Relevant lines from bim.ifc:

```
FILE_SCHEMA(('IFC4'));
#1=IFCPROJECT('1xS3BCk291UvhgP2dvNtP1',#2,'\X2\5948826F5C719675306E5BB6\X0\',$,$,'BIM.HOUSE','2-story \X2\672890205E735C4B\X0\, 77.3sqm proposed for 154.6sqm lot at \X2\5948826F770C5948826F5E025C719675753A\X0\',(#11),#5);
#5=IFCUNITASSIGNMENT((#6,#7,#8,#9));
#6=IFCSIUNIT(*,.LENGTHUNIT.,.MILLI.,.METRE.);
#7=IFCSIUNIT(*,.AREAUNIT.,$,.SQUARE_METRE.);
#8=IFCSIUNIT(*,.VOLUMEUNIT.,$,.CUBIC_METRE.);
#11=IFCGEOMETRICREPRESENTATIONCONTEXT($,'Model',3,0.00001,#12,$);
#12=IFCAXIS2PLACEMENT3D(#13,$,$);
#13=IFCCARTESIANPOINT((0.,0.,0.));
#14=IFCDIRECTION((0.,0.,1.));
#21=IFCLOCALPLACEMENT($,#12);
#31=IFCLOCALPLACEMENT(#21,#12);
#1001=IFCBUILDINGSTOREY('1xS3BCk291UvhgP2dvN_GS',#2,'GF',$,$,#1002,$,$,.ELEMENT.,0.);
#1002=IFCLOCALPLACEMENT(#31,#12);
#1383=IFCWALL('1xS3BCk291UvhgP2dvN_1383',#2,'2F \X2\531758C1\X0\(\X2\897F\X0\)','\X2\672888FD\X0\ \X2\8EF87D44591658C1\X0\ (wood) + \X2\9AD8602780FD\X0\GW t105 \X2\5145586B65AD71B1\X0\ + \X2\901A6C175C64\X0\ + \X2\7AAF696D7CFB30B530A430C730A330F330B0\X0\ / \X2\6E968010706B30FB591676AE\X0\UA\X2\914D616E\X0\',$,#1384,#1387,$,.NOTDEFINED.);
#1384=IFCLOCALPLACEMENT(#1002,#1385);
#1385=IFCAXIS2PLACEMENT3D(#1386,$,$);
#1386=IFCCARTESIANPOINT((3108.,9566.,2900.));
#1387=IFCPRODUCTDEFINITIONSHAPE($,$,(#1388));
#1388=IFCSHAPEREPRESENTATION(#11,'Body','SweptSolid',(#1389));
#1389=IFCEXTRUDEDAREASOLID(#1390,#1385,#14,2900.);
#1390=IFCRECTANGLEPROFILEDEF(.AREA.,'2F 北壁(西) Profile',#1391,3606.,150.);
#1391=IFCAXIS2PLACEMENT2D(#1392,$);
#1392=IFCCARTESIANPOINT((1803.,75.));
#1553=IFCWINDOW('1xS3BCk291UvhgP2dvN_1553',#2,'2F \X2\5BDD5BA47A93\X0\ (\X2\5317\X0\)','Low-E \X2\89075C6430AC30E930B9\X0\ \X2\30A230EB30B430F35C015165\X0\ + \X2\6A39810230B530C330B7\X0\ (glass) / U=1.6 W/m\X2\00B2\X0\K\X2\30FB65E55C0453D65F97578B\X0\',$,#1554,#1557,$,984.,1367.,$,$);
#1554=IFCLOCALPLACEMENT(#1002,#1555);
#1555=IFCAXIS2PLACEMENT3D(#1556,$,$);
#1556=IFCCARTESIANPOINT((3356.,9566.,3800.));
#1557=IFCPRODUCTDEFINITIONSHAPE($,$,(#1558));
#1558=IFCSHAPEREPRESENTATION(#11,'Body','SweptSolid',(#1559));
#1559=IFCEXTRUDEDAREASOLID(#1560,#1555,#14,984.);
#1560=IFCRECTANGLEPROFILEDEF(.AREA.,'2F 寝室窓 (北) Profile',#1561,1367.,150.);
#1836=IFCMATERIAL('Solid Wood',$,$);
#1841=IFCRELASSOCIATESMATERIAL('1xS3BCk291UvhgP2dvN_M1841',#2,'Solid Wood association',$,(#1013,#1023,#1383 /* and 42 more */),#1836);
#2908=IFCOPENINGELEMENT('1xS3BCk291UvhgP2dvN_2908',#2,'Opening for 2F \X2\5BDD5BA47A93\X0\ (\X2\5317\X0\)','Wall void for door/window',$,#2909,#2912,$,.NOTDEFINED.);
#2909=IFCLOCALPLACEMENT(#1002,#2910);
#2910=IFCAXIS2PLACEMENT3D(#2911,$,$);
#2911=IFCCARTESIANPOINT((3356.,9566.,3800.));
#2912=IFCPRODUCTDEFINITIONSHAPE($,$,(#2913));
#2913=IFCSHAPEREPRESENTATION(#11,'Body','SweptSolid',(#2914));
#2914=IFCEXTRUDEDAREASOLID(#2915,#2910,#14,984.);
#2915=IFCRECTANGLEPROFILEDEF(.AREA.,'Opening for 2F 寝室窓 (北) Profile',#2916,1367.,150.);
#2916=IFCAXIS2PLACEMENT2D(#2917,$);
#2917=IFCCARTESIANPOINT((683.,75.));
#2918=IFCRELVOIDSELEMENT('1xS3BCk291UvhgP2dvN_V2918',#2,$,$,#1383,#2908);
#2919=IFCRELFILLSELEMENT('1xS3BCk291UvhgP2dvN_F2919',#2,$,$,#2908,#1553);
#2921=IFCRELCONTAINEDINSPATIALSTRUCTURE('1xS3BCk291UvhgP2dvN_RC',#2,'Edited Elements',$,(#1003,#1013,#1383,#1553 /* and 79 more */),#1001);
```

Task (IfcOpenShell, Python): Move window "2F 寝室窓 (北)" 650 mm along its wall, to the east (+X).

```python
import ifcopenshell
import ifcopenshell.api.geometry
import ifcopenshell.util.placement

model = ifcopenshell.open("bim.ifc")

window = model.by_guid("1xS3BCk291UvhgP2dvN_1553")
opening = window.FillsVoids[0].RelatingOpeningElement
wall = opening.VoidsElements[0].RelatingBuildingElement

wall_matrix = ifcopenshell.util.placement.get_local_placement(wall.ObjectPlacement)
shift = wall_matrix[:3, 0] * 650.0
before = ifcopenshell.util.placement.get_local_placement(window.ObjectPlacement)[:3, 3].copy()

# The window is not placed relative to its opening, so move both.
for product in (opening, window):
    matrix = ifcopenshell.util.placement.get_local_placement(product.ObjectPlacement)
    matrix[:3, 3] += shift
    ifcopenshell.api.geometry.edit_object_placement(model, product=product, matrix=matrix, is_si=False)

after = ifcopenshell.util.placement.get_local_placement(window.ObjectPlacement)[:3, 3]
print("window moved by", (after - before).round(3) + 0.0)

model.write("bim_edited.ifc")
```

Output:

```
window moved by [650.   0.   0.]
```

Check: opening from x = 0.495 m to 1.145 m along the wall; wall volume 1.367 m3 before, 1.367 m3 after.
